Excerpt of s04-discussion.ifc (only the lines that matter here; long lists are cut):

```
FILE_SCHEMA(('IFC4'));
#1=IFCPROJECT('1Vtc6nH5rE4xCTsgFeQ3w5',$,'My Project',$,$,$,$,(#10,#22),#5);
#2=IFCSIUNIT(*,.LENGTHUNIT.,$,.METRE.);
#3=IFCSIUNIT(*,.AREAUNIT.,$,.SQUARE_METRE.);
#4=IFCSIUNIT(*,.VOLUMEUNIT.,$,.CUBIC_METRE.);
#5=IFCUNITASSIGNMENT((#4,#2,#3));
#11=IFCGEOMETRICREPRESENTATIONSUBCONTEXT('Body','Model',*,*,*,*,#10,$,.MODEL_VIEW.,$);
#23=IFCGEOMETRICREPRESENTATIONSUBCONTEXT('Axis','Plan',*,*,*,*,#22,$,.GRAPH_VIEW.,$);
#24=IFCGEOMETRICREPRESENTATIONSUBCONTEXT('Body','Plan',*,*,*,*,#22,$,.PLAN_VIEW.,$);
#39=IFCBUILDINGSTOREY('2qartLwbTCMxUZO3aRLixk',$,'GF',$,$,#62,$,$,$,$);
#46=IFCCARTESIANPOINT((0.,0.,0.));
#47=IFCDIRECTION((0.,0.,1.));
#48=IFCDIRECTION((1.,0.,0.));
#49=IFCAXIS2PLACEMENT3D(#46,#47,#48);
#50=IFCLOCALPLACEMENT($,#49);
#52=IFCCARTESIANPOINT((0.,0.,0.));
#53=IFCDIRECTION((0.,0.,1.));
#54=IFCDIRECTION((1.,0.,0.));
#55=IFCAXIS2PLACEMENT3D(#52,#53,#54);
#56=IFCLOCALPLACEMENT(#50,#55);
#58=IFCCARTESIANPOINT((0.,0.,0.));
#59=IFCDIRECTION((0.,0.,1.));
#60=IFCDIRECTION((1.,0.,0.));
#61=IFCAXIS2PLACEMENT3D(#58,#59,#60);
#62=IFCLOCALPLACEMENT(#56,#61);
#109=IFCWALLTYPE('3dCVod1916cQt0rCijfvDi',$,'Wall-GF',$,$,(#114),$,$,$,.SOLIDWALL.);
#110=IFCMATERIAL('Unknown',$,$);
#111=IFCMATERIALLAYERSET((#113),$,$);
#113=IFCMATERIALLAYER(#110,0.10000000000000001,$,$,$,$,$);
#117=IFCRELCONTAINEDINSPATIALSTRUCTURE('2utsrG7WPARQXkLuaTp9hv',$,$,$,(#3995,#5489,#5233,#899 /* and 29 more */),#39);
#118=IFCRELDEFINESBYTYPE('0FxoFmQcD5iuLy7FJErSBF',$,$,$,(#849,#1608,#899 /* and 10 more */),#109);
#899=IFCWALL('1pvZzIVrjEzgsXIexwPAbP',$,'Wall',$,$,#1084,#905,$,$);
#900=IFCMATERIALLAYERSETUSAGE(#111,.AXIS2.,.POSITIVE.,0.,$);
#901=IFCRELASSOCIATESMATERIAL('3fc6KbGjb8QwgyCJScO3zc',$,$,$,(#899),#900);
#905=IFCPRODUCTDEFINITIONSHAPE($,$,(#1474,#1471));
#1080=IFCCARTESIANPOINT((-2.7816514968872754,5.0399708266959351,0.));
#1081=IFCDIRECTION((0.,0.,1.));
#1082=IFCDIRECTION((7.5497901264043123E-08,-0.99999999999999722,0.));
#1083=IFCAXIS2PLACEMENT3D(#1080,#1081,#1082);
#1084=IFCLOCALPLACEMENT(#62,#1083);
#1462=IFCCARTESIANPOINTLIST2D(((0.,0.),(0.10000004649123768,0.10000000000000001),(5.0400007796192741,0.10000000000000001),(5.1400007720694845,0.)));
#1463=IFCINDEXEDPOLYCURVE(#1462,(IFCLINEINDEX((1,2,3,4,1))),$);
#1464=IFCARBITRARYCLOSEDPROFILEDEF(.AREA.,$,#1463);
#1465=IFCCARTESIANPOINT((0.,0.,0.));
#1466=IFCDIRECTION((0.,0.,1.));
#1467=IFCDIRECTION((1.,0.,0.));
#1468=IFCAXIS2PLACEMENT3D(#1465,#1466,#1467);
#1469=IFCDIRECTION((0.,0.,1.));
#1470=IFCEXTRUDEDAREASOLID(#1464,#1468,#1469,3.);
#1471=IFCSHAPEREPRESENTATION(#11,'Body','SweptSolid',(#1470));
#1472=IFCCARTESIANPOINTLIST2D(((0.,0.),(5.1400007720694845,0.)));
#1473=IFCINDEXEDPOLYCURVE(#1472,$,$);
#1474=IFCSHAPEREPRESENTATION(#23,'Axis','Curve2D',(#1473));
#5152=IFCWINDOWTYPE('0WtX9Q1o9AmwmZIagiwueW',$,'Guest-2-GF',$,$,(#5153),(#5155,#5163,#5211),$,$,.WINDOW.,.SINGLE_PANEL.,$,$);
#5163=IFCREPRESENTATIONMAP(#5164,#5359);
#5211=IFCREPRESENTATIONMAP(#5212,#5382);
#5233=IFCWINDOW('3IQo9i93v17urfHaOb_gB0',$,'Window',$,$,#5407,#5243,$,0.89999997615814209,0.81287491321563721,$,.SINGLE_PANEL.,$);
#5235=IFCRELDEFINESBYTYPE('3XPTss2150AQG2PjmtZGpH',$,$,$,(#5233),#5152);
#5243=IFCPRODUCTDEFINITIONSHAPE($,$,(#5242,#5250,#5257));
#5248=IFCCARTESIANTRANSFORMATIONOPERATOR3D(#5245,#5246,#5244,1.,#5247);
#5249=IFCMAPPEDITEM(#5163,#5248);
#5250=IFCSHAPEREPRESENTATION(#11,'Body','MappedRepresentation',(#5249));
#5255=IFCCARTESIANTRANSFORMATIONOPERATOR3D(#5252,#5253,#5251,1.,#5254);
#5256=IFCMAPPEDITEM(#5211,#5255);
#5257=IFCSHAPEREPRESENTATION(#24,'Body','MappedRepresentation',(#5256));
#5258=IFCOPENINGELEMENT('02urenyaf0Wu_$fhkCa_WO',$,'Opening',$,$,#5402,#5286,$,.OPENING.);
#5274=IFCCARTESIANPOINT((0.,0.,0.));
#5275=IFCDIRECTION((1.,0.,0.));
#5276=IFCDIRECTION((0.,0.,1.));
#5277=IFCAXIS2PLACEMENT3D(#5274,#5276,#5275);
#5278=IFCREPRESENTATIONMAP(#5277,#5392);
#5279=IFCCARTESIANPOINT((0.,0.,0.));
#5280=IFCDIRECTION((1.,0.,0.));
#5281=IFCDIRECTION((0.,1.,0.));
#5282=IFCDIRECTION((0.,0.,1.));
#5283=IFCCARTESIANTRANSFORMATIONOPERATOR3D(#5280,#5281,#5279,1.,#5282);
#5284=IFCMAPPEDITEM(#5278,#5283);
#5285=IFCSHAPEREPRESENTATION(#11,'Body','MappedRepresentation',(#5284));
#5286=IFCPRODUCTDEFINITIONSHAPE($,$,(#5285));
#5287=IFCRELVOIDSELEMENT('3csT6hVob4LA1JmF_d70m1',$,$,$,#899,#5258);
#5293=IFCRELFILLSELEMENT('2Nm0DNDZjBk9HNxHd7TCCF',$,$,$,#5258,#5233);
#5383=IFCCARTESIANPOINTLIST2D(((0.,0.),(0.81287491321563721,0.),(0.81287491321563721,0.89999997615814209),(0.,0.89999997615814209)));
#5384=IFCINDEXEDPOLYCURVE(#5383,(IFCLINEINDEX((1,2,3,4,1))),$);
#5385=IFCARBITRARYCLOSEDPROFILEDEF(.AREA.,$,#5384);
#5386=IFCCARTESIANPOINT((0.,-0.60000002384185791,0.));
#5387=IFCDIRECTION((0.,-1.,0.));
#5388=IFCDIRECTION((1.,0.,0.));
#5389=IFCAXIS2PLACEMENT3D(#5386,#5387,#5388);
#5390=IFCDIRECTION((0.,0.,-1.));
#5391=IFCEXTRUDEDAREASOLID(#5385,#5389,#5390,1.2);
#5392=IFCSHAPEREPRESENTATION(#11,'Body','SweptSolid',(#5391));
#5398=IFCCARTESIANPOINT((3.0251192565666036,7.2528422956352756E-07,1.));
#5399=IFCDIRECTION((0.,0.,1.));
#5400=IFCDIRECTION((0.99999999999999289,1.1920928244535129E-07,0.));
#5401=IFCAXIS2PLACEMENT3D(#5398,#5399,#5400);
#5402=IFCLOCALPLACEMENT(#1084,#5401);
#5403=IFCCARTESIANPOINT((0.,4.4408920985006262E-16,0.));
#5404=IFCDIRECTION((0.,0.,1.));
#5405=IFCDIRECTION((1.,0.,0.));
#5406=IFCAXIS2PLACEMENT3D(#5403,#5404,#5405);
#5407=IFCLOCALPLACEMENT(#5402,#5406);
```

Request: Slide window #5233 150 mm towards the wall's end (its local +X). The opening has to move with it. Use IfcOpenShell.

```python
import ifcopenshell
import ifcopenshell.api.geometry
import ifcopenshell.util.placement
import ifcopenshell.util.unit

model = ifcopenshell.open("s04-discussion.ifc")
unit_scale = ifcopenshell.util.unit.calculate_unit_scale(model)

window = model.by_guid("3IQo9i93v17urfHaOb_gB0")
opening = window.FillsVoids[0].RelatingOpeningElement
wall = opening.VoidsElements[0].RelatingBuildingElement

wall_matrix = ifcopenshell.util.placement.get_local_placement(wall.ObjectPlacement)
shift = wall_matrix[:3, 0] * 0.15 / unit_scale
before = ifcopenshell.util.placement.get_local_placement(window.ObjectPlacement)[:3, 3].copy()

# The window is placed relative to its opening, so it follows when the opening moves.
matrix = ifcopenshell.util.placement.get_local_placement(opening.ObjectPlacement)
matrix[:3, 3] += shift
ifcopenshell.api.geometry.edit_object_placement(
    model, product=opening, matrix=matrix, is_si=False, should_transform_children=True
)

after = ifcopenshell.util.placement.get_local_placement(window.ObjectPlacement)[:3, 3]
print("window moved by", (after - before).round(3) + 0.0)

model.write("s04-discussion_updated.ifc")
```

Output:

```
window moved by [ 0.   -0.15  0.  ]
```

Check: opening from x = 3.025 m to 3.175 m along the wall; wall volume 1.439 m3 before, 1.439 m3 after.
